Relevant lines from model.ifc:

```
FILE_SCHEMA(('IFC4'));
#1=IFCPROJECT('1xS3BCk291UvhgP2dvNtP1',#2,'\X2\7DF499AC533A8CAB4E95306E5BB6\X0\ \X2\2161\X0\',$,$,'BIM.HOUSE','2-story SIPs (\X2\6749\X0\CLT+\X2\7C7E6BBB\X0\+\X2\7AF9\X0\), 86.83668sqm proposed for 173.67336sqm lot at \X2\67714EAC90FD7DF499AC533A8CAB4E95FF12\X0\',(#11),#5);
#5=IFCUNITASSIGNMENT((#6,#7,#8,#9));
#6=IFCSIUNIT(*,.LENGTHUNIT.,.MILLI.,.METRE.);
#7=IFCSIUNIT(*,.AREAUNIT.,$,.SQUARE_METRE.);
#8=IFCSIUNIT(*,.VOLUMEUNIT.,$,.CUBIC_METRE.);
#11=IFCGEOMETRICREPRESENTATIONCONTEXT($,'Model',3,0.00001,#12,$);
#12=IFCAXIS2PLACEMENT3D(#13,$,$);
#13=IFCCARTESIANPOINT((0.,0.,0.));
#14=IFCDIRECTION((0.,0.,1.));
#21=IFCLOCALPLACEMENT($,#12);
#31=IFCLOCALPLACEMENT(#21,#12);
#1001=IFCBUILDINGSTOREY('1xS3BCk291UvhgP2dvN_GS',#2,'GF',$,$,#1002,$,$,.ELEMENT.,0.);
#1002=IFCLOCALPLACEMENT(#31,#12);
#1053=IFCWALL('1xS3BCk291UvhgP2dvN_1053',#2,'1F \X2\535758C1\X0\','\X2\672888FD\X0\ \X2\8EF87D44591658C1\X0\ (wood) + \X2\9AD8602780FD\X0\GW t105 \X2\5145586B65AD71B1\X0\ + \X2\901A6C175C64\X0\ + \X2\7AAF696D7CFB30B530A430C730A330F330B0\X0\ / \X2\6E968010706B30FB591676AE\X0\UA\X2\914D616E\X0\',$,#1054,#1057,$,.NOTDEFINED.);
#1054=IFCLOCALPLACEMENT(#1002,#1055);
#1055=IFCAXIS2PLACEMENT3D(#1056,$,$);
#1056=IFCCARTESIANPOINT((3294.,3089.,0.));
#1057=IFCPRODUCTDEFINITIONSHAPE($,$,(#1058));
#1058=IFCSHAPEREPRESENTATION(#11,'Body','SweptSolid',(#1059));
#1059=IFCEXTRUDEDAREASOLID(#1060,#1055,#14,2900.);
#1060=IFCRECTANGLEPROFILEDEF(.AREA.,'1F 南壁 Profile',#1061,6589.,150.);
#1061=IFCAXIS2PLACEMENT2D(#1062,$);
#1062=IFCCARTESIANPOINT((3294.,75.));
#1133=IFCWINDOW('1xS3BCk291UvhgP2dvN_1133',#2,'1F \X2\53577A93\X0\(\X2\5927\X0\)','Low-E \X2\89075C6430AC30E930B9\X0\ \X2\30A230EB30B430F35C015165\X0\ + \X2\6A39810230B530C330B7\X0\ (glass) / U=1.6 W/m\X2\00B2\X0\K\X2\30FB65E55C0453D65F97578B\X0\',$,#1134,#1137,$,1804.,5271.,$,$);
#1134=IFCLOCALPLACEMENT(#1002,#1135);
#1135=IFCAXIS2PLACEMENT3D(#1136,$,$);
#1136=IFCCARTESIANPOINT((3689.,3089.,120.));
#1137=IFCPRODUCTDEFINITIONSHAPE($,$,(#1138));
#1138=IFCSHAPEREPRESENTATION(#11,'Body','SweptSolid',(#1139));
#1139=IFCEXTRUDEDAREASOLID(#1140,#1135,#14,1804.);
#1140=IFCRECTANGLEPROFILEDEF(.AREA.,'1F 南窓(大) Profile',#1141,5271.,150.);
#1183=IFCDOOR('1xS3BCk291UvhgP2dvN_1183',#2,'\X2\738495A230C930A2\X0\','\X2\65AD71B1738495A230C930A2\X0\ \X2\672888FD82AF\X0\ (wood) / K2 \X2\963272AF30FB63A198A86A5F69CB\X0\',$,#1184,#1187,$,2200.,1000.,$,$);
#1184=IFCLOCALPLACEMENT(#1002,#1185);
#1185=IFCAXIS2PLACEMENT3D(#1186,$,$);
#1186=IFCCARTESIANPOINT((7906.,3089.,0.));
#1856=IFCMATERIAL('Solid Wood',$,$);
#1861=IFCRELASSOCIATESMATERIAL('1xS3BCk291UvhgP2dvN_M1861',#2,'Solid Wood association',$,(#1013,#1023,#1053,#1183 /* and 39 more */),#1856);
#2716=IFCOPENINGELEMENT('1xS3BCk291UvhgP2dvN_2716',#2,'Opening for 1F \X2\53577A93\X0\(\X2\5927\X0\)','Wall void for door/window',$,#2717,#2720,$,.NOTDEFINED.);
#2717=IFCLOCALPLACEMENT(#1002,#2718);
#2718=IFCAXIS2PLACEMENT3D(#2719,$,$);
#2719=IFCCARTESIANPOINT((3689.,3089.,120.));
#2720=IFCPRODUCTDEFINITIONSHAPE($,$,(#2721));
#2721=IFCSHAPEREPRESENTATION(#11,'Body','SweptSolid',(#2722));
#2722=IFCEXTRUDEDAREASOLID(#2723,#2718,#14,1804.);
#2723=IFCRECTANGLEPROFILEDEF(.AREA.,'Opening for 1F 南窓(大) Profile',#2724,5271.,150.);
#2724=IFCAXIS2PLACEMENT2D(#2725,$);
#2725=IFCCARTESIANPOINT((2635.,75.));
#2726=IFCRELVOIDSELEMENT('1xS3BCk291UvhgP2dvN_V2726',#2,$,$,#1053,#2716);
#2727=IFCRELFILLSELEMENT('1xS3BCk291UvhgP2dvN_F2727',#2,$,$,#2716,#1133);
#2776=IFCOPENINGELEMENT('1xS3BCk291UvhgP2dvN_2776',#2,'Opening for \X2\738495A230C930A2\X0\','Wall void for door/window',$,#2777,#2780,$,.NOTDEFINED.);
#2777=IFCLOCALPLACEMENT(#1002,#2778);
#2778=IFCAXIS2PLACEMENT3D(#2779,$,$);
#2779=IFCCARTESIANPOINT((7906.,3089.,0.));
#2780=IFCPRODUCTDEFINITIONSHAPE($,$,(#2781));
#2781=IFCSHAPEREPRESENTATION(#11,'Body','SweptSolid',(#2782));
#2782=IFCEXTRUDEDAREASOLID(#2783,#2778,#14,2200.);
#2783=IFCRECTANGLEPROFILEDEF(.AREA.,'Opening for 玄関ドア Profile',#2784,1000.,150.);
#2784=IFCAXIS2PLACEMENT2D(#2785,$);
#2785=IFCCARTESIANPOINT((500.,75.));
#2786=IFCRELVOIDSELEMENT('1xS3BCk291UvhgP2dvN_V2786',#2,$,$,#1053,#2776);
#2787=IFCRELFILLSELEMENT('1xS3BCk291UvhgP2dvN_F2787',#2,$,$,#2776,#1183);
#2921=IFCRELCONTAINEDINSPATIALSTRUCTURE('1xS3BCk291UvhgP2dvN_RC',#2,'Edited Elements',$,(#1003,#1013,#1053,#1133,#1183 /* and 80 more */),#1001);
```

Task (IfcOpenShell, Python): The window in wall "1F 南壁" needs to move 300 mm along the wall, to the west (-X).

```python
import ifcopenshell
import ifcopenshell.api.geometry
import ifcopenshell.util.placement
import ifcopenshell.util.unit

model = ifcopenshell.open("model.ifc")
unit_scale = ifcopenshell.util.unit.calculate_unit_scale(model)

window = model.by_guid("1xS3BCk291UvhgP2dvN_1133")
opening = window.FillsVoids[0].RelatingOpeningElement
wall = opening.VoidsElements[0].RelatingBuildingElement

wall_matrix = ifcopenshell.util.placement.get_local_placement(wall.ObjectPlacement)
shift = wall_matrix[:3, 0] * -0.3 / unit_scale
before = ifcopenshell.util.placement.get_local_placement(window.ObjectPlacement)[:3, 3].copy()

# The window is not placed relative to its opening, so move both.
for product in (opening, window):
    matrix = ifcopenshell.util.placement.get_local_placement(product.ObjectPlacement)
    matrix[:3, 3] += shift
    ifcopenshell.api.geometry.edit_object_placement(model, product=product, matrix=matrix, is_si=False)

after = ifcopenshell.util.placement.get_local_placement(window.ObjectPlacement)[:3, 3]
print("window moved by", (after - before).round(3) + 0.0)

model.write("model_rev.ifc")
```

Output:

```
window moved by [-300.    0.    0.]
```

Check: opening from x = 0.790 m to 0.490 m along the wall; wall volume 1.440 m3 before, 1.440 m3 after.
